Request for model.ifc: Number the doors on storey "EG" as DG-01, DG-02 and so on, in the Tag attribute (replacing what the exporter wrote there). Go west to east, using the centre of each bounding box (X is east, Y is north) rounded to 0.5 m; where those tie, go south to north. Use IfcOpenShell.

First a look at what the model holds.

```python
import ifcopenshell
import ifcopenshell.util.element
import ifcopenshell.util.placement

model = ifcopenshell.open("model.ifc")
print(model.schema)
storey = next(s for s in model.by_type("IfcBuildingStorey") if s.Name == "EG")
doors = [e for e in ifcopenshell.util.element.get_decomposition(storey) if e.is_a("IfcDoor")]
for e in sorted(doors, key=lambda e: e.id()):
    origin = ifcopenshell.util.placement.get_local_placement(e.ObjectPlacement)[:3, 3]
    print(e.id(), e.Tag, e.Name, origin.round(2) + 0.0, sep=" | ")
```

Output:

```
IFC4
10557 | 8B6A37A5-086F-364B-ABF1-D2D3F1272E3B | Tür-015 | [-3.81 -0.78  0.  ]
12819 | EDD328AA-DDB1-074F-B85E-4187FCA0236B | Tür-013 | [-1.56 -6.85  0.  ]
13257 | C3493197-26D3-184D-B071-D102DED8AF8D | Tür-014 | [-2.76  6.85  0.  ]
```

```python
import ifcopenshell
import ifcopenshell.geom
import ifcopenshell.util.element
import ifcopenshell.util.shape

model = ifcopenshell.open("model.ifc")
settings = ifcopenshell.geom.settings()
settings.set("use-world-coords", True)


def centre(element):
    shape = ifcopenshell.geom.create_shape(settings, element)
    return ifcopenshell.util.shape.get_bbox_centroid(shape.geometry)


storey = next(s for s in model.by_type("IfcBuildingStorey") if s.Name == "EG")
doors = [e for e in ifcopenshell.util.element.get_decomposition(storey) if e.is_a("IfcDoor")]

# Insertion points can sit at a corner or the storey origin, so sort by the geometry (in metres).
centres = {e: centre(e) for e in doors}
doors.sort(key=lambda e: (round(centres[e][0] / 0.5), centres[e][1]))

for i, e in enumerate(doors, start=1):
    number = f"DG-{i:02d}"
    e.Tag = number
    print(e.id(), number)

model.write("model_rev.ifc")
```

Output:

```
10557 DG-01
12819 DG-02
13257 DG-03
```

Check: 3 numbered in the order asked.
